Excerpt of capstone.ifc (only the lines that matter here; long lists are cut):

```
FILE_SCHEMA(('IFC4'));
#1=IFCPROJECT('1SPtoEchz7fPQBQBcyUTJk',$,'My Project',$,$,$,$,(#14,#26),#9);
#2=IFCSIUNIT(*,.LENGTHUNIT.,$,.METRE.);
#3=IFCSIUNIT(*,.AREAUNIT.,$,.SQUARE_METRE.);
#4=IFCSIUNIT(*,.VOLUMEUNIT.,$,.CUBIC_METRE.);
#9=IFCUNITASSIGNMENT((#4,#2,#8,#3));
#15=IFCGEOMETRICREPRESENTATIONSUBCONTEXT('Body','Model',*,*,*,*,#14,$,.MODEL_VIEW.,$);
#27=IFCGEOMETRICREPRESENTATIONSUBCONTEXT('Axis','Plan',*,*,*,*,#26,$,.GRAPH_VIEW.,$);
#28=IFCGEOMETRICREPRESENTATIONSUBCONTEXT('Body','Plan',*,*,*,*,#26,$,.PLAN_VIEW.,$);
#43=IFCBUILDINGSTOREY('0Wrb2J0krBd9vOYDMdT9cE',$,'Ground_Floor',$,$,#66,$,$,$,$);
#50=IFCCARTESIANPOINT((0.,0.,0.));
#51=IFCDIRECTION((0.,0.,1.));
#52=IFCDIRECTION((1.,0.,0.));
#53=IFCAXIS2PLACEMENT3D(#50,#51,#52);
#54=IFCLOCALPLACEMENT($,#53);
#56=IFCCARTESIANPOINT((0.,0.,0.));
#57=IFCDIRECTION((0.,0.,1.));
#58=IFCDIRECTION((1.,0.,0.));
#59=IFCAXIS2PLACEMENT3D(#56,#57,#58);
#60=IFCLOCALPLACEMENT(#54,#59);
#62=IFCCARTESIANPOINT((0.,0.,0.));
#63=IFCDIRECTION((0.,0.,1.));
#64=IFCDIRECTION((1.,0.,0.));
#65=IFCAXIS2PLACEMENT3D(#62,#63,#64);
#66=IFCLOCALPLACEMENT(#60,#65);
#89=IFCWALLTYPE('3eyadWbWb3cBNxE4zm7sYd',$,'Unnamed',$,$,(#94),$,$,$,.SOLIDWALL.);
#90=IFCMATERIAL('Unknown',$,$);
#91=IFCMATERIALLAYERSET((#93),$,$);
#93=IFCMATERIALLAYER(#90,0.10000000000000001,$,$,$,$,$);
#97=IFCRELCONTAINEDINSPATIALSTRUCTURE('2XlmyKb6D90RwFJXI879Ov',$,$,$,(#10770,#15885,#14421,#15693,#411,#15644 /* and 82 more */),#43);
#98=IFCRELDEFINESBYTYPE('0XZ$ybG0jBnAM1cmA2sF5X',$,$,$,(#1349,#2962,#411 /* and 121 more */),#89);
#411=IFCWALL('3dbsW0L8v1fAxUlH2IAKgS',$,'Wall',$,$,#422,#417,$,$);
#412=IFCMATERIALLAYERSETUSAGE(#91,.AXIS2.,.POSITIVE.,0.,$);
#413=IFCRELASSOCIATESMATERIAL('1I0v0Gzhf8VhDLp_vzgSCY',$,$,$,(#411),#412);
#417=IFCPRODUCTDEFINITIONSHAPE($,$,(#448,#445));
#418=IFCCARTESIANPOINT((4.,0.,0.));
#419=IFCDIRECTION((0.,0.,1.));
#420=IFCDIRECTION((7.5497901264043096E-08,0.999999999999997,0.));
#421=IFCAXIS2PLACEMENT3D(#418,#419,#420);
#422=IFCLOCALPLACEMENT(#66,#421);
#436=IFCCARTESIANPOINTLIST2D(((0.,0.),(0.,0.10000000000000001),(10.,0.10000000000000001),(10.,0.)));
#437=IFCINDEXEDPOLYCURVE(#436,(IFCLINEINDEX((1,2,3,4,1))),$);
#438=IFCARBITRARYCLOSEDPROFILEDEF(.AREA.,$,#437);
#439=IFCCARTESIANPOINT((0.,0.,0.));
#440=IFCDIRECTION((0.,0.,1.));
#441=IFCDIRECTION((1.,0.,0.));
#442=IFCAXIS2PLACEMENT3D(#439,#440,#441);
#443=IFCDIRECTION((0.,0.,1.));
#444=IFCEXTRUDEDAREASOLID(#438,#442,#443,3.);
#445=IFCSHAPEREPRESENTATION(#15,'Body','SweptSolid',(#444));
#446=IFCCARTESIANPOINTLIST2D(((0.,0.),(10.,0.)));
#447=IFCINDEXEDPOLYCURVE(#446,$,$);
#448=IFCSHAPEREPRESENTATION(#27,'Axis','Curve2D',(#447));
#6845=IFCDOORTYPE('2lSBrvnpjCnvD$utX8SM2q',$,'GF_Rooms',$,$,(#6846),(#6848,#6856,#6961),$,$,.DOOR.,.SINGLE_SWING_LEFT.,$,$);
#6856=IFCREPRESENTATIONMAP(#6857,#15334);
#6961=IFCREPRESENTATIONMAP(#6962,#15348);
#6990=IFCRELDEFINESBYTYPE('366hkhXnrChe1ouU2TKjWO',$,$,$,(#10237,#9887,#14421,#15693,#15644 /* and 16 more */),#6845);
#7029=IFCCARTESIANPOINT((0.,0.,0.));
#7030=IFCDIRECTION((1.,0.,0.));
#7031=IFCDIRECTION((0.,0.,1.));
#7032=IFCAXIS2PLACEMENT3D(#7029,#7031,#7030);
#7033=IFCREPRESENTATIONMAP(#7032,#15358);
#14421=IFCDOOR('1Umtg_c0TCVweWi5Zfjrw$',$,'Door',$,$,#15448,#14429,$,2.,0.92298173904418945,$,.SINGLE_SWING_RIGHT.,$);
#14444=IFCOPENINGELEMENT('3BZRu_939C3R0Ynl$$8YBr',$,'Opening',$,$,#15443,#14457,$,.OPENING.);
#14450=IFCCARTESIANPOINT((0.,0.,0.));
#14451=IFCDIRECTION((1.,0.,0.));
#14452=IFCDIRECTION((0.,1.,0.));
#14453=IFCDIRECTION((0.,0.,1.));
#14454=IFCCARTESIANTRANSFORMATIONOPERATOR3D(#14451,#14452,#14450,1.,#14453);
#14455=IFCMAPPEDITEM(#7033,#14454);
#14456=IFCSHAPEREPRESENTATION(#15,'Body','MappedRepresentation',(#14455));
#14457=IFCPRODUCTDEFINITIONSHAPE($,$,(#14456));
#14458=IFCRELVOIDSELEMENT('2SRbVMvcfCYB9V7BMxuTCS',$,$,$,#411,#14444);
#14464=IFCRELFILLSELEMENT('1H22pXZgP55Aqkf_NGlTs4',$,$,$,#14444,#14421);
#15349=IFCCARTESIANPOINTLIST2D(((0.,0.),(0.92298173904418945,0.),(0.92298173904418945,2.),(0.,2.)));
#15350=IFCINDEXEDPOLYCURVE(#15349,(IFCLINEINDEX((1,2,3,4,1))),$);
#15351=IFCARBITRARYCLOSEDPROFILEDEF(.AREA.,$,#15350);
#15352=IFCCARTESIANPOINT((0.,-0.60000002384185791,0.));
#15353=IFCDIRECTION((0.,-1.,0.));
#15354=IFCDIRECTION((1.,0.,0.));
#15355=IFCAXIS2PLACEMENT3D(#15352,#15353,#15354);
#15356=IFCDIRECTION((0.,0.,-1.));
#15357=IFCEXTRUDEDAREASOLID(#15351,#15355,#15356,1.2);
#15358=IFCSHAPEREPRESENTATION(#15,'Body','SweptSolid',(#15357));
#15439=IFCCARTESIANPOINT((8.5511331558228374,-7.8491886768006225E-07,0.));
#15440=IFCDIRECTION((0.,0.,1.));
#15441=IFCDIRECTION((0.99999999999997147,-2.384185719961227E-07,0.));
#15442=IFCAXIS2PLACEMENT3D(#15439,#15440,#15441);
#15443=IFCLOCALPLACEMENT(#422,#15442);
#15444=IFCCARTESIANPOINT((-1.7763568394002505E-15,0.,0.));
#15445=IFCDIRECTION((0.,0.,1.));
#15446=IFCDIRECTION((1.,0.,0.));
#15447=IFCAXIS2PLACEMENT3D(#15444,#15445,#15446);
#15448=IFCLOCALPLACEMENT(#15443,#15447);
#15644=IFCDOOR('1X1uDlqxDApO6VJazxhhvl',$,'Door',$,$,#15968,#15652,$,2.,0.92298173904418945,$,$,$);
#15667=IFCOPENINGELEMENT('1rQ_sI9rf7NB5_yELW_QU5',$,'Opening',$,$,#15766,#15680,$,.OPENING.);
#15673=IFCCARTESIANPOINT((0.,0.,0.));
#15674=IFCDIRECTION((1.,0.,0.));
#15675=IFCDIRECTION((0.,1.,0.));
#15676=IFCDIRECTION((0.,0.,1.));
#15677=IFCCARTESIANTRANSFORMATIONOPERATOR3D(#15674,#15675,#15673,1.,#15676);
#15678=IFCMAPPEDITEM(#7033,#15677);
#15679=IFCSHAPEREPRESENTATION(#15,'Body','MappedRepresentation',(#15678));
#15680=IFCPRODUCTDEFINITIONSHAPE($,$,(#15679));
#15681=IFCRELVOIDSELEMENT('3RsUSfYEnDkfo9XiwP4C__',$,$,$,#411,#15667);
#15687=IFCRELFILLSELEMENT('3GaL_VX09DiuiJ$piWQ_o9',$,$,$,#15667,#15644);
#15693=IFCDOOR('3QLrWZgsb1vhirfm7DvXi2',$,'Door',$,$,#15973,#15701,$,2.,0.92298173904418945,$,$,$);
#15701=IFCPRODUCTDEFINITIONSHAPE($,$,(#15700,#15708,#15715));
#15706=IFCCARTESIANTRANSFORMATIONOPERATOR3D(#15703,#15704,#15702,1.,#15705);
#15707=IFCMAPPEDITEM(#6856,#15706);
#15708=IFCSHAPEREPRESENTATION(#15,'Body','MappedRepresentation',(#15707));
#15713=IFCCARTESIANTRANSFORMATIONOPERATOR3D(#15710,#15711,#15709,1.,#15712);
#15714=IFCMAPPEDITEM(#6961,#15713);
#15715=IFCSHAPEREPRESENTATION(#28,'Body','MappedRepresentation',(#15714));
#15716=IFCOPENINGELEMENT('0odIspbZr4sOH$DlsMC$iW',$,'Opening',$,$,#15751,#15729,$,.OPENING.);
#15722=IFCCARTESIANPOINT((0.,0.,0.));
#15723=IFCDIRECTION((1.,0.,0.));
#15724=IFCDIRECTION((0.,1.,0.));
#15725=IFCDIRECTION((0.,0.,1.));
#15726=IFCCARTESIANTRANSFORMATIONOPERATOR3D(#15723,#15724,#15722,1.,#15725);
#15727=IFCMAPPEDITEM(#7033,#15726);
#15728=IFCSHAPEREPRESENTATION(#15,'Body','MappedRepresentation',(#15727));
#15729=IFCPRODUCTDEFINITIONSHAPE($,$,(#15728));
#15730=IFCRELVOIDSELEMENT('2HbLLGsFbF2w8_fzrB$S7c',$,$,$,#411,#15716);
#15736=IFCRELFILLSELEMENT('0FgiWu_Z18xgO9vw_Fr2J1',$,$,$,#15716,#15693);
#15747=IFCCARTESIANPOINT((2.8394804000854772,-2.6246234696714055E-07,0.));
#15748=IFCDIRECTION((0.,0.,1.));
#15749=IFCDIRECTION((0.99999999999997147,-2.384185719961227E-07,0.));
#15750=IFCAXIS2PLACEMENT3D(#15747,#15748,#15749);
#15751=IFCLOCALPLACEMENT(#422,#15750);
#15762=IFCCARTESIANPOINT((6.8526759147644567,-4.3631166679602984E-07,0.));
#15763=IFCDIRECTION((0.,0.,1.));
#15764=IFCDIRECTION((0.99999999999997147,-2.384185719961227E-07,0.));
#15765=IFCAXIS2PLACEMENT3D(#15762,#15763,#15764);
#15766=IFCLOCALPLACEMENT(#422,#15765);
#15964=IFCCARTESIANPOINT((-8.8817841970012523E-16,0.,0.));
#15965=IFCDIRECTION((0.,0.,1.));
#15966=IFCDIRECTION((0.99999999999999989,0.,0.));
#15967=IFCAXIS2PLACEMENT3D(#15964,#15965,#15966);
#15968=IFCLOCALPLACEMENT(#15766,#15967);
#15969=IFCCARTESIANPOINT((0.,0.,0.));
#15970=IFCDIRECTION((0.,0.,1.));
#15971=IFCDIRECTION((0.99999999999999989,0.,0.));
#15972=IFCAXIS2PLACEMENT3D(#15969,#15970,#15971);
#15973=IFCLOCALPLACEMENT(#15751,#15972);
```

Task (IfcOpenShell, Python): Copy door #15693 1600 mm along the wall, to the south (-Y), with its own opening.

```python
import ifcopenshell
import ifcopenshell.api.feature
import ifcopenshell.api.geometry
import ifcopenshell.api.root
import ifcopenshell.geom
import ifcopenshell.util.element
import ifcopenshell.util.placement
import ifcopenshell.util.shape
import ifcopenshell.util.unit

model = ifcopenshell.open("capstone.ifc")
unit_scale = ifcopenshell.util.unit.calculate_unit_scale(model)
settings = ifcopenshell.geom.settings()


def volume(element):
    """Net volume in cubic metres, openings subtracted."""
    shape = ifcopenshell.geom.create_shape(settings, element)
    return ifcopenshell.util.shape.get_volume(shape.geometry)


door = model.by_guid("3QLrWZgsb1vhirfm7DvXi2")
opening = door.FillsVoids[0].RelatingOpeningElement
wall = opening.VoidsElements[0].RelatingBuildingElement
before = volume(wall)
shift = ifcopenshell.util.placement.get_local_placement(wall.ObjectPlacement)[:3, 0] * -1.6 / unit_scale

# copy_class copies the void relationship, type, container and properties, but no geometry.
new_opening = ifcopenshell.api.root.copy_class(model, product=opening)
new_opening.Representation = ifcopenshell.util.element.copy_deep(
    model, opening.Representation, exclude=["IfcGeometricRepresentationContext", "IfcRepresentationMap"]
)
new_door = ifcopenshell.api.root.copy_class(model, product=door)
new_door.Representation = ifcopenshell.util.element.copy_deep(
    model, door.Representation, exclude=["IfcGeometricRepresentationContext", "IfcRepresentationMap"]
)
ifcopenshell.api.feature.add_filling(model, opening=new_opening, element=new_door)

for old, new in ((opening, new_opening), (door, new_door)):
    matrix = ifcopenshell.util.placement.get_local_placement(old.ObjectPlacement)
    matrix[:3, 3] += shift
    ifcopenshell.api.geometry.edit_object_placement(model, product=new, matrix=matrix, is_si=False)

after = volume(wall)

print(f"wall volume {before:.3f} -> {after:.3f} m3")

model.write("capstone_v2.ifc")
```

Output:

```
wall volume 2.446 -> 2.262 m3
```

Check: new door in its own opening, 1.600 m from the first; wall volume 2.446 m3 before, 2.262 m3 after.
